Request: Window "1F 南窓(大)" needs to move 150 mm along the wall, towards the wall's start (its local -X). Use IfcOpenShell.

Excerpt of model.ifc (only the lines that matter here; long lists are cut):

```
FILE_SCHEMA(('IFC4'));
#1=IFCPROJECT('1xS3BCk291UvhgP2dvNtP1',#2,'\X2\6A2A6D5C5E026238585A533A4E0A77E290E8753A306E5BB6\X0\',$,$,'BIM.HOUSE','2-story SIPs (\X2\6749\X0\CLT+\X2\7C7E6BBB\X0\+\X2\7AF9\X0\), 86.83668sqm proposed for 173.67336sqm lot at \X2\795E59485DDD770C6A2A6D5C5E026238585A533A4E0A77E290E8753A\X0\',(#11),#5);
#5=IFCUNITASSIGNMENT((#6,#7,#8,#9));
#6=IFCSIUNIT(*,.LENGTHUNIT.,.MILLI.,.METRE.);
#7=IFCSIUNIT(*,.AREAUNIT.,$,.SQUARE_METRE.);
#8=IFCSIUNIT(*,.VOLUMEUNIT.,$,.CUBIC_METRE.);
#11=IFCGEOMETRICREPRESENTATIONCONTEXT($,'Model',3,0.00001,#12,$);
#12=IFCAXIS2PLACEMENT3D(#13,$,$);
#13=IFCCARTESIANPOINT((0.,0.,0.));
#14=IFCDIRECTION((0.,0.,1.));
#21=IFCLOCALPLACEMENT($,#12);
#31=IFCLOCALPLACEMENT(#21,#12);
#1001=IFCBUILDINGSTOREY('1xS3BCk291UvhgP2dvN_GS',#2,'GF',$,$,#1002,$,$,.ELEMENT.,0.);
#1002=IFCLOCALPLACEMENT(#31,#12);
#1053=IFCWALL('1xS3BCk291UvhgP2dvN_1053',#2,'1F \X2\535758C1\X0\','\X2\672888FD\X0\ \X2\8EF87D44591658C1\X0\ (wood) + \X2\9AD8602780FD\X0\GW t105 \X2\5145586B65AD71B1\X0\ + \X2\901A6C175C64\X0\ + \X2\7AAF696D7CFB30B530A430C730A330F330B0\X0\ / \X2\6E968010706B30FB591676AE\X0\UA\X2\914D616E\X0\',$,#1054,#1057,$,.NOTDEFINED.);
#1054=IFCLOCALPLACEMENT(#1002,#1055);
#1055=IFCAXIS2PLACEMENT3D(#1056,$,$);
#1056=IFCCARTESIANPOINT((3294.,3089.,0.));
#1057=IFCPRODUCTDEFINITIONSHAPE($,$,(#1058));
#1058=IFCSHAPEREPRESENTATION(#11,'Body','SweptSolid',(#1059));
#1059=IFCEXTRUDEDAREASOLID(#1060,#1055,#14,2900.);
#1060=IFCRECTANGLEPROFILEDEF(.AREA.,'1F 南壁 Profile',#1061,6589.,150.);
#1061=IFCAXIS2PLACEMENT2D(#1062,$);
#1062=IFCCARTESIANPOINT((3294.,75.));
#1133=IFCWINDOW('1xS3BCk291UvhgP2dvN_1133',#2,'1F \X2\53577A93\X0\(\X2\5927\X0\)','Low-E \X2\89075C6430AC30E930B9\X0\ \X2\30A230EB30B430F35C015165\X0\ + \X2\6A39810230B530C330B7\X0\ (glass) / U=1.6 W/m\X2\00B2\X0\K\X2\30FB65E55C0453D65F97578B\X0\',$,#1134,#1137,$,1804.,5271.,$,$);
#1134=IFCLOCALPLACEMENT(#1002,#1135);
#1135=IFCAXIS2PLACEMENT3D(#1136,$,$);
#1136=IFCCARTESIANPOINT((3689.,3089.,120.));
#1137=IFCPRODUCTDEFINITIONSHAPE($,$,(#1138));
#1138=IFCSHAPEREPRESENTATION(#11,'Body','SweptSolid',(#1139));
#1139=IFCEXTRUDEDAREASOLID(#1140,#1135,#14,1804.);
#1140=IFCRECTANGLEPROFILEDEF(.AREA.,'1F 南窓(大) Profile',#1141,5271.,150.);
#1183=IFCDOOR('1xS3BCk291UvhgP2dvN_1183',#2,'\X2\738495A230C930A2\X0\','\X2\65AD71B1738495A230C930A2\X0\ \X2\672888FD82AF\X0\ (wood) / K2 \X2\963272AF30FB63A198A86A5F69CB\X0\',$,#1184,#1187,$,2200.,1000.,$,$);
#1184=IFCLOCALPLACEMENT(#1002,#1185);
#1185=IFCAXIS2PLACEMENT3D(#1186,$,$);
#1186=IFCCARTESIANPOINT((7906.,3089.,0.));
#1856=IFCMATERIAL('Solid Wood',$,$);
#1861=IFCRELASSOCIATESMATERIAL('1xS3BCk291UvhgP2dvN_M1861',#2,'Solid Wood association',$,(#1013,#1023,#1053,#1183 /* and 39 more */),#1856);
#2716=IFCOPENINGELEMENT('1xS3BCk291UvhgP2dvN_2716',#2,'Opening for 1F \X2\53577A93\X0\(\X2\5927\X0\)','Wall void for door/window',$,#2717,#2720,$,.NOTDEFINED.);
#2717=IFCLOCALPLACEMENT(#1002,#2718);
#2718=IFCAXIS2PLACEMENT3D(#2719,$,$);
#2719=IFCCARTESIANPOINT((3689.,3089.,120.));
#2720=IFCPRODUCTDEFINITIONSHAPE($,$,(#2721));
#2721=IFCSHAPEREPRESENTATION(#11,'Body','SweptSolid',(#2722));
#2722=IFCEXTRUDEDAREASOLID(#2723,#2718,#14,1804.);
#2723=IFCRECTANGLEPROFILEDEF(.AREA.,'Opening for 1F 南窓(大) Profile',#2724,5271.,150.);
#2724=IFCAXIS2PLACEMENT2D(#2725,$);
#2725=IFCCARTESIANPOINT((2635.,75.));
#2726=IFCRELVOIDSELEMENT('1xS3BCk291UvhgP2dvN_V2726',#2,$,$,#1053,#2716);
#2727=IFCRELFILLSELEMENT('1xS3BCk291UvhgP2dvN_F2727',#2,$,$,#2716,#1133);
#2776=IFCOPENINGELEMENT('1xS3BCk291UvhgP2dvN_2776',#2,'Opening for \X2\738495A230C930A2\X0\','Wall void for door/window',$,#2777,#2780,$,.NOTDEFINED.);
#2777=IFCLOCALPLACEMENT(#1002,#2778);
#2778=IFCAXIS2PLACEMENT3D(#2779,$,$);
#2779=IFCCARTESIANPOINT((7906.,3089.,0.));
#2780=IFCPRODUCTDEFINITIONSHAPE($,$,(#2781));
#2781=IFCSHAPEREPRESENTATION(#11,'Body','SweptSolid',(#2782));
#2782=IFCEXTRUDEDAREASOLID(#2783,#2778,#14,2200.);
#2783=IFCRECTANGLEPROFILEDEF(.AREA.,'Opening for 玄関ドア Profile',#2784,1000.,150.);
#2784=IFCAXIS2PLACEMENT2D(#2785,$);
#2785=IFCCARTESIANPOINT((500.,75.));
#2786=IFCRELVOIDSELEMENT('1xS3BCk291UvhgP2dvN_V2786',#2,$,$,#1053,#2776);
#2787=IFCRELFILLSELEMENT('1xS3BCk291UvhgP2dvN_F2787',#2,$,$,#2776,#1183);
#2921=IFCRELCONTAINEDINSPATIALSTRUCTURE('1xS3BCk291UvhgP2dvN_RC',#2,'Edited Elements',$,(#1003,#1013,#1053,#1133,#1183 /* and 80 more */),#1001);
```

```python
import ifcopenshell
import ifcopenshell.api.geometry
import ifcopenshell.util.placement

model = ifcopenshell.open("model.ifc")

window = model.by_guid("1xS3BCk291UvhgP2dvN_1133")
opening = window.FillsVoids[0].RelatingOpeningElement
wall = opening.VoidsElements[0].RelatingBuildingElement

wall_matrix = ifcopenshell.util.placement.get_local_placement(wall.ObjectPlacement)
shift = wall_matrix[:3, 0] * -150.0
before = ifcopenshell.util.placement.get_local_placement(window.ObjectPlacement)[:3, 3].copy()

# The window is not placed relative to its opening, so move both.
for product in (opening, window):
    matrix = ifcopenshell.util.placement.get_local_placement(product.ObjectPlacement)
    matrix[:3, 3] += shift
    ifcopenshell.api.geometry.edit_object_placement(model, product=product, matrix=matrix, is_si=False)

after = ifcopenshell.util.placement.get_local_placement(window.ObjectPlacement)[:3, 3]
print("window moved by", (after - before).round(3) + 0.0)

model.write("model_edited.ifc")
```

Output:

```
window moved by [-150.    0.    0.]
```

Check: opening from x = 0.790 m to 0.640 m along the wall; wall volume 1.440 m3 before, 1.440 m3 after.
